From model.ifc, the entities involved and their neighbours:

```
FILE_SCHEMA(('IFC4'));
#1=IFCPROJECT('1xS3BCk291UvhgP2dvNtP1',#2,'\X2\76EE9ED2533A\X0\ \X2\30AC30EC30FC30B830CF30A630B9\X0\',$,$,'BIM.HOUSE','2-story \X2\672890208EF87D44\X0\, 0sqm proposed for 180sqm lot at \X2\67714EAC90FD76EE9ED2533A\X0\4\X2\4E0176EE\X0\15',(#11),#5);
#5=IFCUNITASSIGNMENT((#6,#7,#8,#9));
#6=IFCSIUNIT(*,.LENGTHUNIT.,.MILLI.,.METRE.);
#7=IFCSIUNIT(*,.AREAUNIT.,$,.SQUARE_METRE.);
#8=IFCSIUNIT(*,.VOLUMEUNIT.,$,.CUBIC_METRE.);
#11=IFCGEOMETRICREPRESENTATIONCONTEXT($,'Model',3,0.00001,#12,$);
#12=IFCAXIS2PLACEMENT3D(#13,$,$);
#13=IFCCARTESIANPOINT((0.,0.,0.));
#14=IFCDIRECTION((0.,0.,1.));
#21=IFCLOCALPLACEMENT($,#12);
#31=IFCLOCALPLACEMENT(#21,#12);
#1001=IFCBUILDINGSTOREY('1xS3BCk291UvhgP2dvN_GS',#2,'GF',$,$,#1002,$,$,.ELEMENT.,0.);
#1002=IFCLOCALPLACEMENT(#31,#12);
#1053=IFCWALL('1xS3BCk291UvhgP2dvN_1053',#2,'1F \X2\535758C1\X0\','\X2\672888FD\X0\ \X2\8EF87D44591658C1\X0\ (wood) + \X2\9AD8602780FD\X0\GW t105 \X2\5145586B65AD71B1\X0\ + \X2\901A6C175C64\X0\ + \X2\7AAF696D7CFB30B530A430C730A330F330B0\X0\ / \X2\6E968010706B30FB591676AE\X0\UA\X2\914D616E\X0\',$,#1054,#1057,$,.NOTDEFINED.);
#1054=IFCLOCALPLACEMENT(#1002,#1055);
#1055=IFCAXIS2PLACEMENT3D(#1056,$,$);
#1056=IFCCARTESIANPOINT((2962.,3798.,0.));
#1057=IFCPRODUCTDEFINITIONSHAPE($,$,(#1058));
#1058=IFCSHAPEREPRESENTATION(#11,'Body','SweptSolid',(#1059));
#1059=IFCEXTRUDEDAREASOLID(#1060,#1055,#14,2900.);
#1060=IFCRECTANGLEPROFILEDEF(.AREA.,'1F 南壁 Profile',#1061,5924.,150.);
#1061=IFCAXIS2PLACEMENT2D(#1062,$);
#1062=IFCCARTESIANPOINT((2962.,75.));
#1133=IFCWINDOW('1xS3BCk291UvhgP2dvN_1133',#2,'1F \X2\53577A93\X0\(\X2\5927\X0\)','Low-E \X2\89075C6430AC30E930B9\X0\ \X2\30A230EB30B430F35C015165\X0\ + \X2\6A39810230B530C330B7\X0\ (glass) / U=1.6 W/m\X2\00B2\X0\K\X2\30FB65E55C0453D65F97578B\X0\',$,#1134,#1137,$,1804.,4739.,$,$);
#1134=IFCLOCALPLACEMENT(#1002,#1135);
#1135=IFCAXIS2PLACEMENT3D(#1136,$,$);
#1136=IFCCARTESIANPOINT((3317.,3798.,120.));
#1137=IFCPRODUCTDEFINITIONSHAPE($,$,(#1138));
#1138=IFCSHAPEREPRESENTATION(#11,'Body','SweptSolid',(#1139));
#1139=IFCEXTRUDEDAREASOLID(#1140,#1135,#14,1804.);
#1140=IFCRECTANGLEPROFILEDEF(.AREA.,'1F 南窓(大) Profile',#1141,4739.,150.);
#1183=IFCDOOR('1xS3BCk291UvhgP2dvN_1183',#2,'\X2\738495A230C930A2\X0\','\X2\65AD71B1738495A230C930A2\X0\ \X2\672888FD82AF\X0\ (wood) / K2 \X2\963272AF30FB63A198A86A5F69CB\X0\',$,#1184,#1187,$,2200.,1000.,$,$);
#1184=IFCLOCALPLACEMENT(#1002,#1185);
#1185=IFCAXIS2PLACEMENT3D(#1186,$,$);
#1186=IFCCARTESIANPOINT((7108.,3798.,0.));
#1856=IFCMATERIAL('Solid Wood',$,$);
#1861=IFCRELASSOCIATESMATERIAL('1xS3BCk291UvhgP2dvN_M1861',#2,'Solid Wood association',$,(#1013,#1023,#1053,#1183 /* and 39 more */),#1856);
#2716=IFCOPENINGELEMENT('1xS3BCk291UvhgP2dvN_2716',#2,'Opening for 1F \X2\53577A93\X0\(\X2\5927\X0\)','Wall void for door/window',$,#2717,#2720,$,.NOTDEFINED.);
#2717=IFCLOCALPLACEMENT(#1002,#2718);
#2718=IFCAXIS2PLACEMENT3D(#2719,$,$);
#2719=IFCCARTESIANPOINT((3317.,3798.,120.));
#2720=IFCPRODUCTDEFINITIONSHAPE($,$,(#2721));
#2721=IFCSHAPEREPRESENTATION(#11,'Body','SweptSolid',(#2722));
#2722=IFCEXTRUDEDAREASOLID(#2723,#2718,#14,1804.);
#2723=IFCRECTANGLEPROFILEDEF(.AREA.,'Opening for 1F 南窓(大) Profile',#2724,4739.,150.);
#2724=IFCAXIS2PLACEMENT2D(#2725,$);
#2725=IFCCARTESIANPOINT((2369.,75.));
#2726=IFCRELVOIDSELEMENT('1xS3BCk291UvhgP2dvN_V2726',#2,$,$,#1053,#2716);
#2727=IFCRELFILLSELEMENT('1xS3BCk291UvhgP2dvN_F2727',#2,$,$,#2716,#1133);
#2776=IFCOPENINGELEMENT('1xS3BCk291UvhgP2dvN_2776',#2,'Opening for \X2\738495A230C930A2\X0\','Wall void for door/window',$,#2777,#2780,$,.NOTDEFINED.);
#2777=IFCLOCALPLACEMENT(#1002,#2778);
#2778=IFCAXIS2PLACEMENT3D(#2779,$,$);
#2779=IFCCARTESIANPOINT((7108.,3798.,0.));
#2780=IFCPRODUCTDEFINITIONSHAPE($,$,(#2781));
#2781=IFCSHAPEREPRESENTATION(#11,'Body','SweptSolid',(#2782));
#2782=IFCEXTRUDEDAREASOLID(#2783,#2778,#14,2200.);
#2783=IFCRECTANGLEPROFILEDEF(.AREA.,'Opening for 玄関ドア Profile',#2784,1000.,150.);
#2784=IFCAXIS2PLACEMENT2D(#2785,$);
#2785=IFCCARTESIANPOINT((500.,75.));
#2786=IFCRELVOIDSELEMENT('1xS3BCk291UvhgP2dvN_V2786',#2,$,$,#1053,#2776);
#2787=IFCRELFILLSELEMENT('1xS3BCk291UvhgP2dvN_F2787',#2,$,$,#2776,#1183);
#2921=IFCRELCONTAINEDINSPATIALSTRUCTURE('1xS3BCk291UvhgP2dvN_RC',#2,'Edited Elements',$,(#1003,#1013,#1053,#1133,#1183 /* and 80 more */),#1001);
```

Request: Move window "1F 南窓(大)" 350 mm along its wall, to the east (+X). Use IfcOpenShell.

```python
import ifcopenshell
import ifcopenshell.api.geometry
import ifcopenshell.util.placement
import ifcopenshell.util.unit

model = ifcopenshell.open("model.ifc")
unit_scale = ifcopenshell.util.unit.calculate_unit_scale(model)

window = model.by_guid("1xS3BCk291UvhgP2dvN_1133")
opening = window.FillsVoids[0].RelatingOpeningElement
wall = opening.VoidsElements[0].RelatingBuildingElement

wall_matrix = ifcopenshell.util.placement.get_local_placement(wall.ObjectPlacement)
shift = wall_matrix[:3, 0] * 0.35 / unit_scale
before = ifcopenshell.util.placement.get_local_placement(window.ObjectPlacement)[:3, 3].copy()

# The window is not placed relative to its opening, so move both.
for product in (opening, window):
    matrix = ifcopenshell.util.placement.get_local_placement(product.ObjectPlacement)
    matrix[:3, 3] += shift
    ifcopenshell.api.geometry.edit_object_placement(model, product=product, matrix=matrix, is_si=False)

after = ifcopenshell.util.placement.get_local_placement(window.ObjectPlacement)[:3, 3]
print("window moved by", (after - before).round(3) + 0.0)

model.write("model-out.ifc")
```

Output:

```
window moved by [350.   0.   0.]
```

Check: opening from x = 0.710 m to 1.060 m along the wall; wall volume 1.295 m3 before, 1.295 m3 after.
